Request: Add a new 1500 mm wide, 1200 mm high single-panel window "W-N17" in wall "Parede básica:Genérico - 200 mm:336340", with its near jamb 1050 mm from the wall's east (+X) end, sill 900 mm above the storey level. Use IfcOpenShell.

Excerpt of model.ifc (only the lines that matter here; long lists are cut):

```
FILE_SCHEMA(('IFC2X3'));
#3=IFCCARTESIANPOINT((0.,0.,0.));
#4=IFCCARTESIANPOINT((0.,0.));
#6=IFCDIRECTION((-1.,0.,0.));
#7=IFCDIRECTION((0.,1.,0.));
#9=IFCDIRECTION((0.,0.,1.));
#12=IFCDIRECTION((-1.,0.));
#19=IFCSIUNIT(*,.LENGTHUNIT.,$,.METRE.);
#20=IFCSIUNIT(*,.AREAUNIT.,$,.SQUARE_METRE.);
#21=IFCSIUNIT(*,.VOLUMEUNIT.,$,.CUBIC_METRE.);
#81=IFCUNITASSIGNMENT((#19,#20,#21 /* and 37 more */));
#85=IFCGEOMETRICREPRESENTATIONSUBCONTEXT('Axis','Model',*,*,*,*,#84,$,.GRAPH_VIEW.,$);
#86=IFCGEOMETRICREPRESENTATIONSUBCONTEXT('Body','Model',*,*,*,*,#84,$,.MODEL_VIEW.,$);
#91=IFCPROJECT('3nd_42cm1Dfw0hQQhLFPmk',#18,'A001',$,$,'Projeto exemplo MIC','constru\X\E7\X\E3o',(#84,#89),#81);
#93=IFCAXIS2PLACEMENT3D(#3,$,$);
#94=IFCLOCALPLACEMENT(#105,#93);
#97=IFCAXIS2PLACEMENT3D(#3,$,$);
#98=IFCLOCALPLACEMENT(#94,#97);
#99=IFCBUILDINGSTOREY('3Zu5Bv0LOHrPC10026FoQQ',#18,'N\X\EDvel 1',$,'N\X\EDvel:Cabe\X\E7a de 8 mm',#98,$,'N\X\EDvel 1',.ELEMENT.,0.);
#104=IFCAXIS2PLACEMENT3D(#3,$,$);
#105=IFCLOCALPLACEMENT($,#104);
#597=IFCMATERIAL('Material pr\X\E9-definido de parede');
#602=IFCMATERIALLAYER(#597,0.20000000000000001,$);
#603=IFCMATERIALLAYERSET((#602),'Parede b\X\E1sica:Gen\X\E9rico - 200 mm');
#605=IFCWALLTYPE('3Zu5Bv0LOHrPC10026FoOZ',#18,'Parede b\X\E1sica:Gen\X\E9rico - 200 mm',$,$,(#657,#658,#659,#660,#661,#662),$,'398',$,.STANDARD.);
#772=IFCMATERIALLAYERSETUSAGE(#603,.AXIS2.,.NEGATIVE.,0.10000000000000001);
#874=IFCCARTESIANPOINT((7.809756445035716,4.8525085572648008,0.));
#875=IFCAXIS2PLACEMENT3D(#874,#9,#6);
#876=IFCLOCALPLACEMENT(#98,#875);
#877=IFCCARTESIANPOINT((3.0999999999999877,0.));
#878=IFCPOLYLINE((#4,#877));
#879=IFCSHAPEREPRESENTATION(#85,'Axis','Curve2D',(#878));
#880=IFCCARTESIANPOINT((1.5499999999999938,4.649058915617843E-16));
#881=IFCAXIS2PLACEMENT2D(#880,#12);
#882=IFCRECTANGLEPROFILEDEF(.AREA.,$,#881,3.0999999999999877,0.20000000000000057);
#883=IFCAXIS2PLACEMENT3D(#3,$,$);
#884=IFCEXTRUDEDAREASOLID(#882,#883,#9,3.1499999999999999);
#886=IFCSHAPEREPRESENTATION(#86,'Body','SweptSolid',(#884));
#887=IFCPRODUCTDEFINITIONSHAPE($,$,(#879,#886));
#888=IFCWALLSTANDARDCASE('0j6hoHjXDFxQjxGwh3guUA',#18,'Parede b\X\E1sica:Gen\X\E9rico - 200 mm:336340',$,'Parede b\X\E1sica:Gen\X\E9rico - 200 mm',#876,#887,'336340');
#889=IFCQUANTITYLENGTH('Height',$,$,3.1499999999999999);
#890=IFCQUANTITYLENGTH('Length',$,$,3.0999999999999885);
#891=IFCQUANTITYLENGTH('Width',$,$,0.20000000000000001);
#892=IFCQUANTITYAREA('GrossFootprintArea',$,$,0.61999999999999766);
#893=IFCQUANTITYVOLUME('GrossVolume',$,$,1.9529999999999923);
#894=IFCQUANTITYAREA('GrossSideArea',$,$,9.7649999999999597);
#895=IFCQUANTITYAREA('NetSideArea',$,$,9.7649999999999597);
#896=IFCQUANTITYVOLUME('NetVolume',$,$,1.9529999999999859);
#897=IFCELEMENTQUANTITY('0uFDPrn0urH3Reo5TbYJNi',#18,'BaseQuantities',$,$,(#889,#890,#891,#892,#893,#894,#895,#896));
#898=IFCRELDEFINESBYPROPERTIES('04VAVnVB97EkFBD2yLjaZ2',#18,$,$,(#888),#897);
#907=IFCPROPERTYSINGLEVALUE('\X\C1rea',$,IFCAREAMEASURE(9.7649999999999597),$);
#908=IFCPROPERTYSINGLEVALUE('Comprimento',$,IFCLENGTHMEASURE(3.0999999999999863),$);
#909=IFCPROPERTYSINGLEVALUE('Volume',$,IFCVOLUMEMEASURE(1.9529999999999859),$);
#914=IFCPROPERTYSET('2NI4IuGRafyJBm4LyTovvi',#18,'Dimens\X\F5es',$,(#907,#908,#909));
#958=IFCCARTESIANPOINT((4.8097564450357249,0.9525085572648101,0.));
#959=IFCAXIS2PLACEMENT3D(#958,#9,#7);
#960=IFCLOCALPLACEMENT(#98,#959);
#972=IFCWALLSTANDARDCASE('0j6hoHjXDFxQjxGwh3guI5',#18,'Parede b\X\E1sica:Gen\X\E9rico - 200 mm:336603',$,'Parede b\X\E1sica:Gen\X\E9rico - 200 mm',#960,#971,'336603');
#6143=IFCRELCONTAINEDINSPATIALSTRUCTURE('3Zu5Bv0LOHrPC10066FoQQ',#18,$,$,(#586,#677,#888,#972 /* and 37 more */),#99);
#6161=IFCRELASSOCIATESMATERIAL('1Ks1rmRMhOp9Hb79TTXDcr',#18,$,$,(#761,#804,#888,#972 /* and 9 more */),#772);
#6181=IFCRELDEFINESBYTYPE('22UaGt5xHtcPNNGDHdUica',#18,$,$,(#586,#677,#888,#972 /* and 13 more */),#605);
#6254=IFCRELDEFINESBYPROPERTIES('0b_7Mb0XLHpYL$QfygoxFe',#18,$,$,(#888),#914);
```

```python
import numpy as np
import ifcopenshell
import ifcopenshell.api.feature
import ifcopenshell.api.geometry
import ifcopenshell.api.pset
import ifcopenshell.api.root
import ifcopenshell.api.spatial
import ifcopenshell.api.type
import ifcopenshell.geom
import ifcopenshell.util.element
import ifcopenshell.util.placement
import ifcopenshell.util.representation
import ifcopenshell.util.shape
import ifcopenshell.util.unit

model = ifcopenshell.open("model.ifc")
unit_scale = ifcopenshell.util.unit.calculate_unit_scale(model)
area_scale = ifcopenshell.util.unit.calculate_unit_scale(model, "AREAUNIT")
volume_scale = ifcopenshell.util.unit.calculate_unit_scale(model, "VOLUMEUNIT")
settings = ifcopenshell.geom.settings()


def volume(element):
    """Net volume in cubic metres, openings subtracted."""
    shape = ifcopenshell.geom.create_shape(settings, element)
    return ifcopenshell.util.shape.get_volume(shape.geometry)


wall = model.by_guid("0j6hoHjXDFxQjxGwh3guUA")
storey = ifcopenshell.util.element.get_container(wall, ifc_class="IfcBuildingStorey")
context = ifcopenshell.util.representation.get_context(model, "Model", "Body", "MODEL_VIEW")
before = volume(wall)

width, height, from_end, sill = 1.5, 1.2, 1.05, 0.9  # metres

# The wall runs along its own X axis, and the end named is its -X end.
wall_shape = ifcopenshell.geom.create_shape(settings, wall)
x, y, z = ifcopenshell.util.shape.get_vertices(wall_shape.geometry).T
start = x.min() + from_end
face, thickness = float(y.min()), float(y.max() - y.min())
wall_matrix = ifcopenshell.util.placement.get_local_placement(wall.ObjectPlacement)
level = ifcopenshell.util.placement.get_local_placement(storey.ObjectPlacement)[2, 3]


def in_wall(x, y):
    """Placement at x, y metres in the wall's axes, at sill height."""
    matrix = wall_matrix.copy()
    matrix[:, 3] = wall_matrix @ np.array([x / unit_scale, y / unit_scale, 0.0, 1.0])
    matrix[2, 3] = level + sill / unit_scale
    return matrix


# Opening: a box that overshoots both wall faces by 50 mm.
opening = ifcopenshell.api.root.create_entity(model, ifc_class="IfcOpeningElement")
box = ifcopenshell.api.geometry.add_wall_representation(
    model, context=context, length=width, height=height, thickness=thickness + 0.1
)
ifcopenshell.api.geometry.assign_representation(model, product=opening, representation=box)
ifcopenshell.api.geometry.edit_object_placement(model, product=opening, matrix=in_wall(start, face - 0.05), is_si=False)
ifcopenshell.api.feature.add_feature(model, feature=opening, element=wall)

window = ifcopenshell.api.root.create_entity(model, ifc_class="IfcWindow", name="W-N17")
window.OverallWidth, window.OverallHeight = width / unit_scale, height / unit_scale
body = ifcopenshell.api.geometry.add_window_representation(
    model,
    context=context,
    overall_width=window.OverallWidth,
    overall_height=window.OverallHeight,
    partition_type="SINGLE_PANEL",
)
ifcopenshell.api.geometry.assign_representation(model, product=window, representation=body)
ifcopenshell.api.spatial.assign_container(model, products=[window], relating_structure=storey)
fills = ifcopenshell.api.feature.add_filling(model, opening=opening, element=window)
fills.OwnerHistory = window.OwnerHistory  # required in IFC2X3

# IFC2X3 keeps the operation on the window style.
style = ifcopenshell.api.root.create_entity(model, ifc_class="IfcWindowStyle", name="W-N17")
style.OperationType, style.ConstructionType = "SINGLE_PANEL", "NOTDEFINED"
style.ParameterTakesPrecedence = style.Sizeable = False
ifcopenshell.api.type.assign_type(model, related_objects=[window], relating_type=style)

# Centre the window in the wall's thickness.
ifcopenshell.api.geometry.edit_object_placement(model, product=window, matrix=in_wall(start, face), is_si=False)
window_shape = ifcopenshell.geom.create_shape(settings, window)
depth = ifcopenshell.util.shape.get_vertices(window_shape.geometry)[:, 1]
offset = face + thickness / 2 - (depth.min() + depth.max()) / 2
ifcopenshell.api.geometry.edit_object_placement(model, product=window, matrix=in_wall(start, offset), is_si=False)

after = volume(wall)

# Update the wall's stored quantities.
qto = model.by_id(ifcopenshell.util.element.get_pset(wall, "BaseQuantities", should_inherit=False)["id"])
ifcopenshell.api.pset.edit_qto(model, qto=qto, properties={
    "NetSideArea": after / thickness / area_scale,
    "NetVolume": after / volume_scale,
})
pset = model.by_id(ifcopenshell.util.element.get_pset(wall, "Dimensões", should_inherit=False)["id"])
ifcopenshell.api.pset.edit_pset(model, pset=pset, properties={
    "Área": model.create_entity("IfcAreaMeasure", after / thickness / area_scale),
    "Volume": model.create_entity("IfcVolumeMeasure", after / volume_scale),
})

print(f"wall volume {before:.3f} -> {after:.3f} m3")

model.write("model-out.ifc")
```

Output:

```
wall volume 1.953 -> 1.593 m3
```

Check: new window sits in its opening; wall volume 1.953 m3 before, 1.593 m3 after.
